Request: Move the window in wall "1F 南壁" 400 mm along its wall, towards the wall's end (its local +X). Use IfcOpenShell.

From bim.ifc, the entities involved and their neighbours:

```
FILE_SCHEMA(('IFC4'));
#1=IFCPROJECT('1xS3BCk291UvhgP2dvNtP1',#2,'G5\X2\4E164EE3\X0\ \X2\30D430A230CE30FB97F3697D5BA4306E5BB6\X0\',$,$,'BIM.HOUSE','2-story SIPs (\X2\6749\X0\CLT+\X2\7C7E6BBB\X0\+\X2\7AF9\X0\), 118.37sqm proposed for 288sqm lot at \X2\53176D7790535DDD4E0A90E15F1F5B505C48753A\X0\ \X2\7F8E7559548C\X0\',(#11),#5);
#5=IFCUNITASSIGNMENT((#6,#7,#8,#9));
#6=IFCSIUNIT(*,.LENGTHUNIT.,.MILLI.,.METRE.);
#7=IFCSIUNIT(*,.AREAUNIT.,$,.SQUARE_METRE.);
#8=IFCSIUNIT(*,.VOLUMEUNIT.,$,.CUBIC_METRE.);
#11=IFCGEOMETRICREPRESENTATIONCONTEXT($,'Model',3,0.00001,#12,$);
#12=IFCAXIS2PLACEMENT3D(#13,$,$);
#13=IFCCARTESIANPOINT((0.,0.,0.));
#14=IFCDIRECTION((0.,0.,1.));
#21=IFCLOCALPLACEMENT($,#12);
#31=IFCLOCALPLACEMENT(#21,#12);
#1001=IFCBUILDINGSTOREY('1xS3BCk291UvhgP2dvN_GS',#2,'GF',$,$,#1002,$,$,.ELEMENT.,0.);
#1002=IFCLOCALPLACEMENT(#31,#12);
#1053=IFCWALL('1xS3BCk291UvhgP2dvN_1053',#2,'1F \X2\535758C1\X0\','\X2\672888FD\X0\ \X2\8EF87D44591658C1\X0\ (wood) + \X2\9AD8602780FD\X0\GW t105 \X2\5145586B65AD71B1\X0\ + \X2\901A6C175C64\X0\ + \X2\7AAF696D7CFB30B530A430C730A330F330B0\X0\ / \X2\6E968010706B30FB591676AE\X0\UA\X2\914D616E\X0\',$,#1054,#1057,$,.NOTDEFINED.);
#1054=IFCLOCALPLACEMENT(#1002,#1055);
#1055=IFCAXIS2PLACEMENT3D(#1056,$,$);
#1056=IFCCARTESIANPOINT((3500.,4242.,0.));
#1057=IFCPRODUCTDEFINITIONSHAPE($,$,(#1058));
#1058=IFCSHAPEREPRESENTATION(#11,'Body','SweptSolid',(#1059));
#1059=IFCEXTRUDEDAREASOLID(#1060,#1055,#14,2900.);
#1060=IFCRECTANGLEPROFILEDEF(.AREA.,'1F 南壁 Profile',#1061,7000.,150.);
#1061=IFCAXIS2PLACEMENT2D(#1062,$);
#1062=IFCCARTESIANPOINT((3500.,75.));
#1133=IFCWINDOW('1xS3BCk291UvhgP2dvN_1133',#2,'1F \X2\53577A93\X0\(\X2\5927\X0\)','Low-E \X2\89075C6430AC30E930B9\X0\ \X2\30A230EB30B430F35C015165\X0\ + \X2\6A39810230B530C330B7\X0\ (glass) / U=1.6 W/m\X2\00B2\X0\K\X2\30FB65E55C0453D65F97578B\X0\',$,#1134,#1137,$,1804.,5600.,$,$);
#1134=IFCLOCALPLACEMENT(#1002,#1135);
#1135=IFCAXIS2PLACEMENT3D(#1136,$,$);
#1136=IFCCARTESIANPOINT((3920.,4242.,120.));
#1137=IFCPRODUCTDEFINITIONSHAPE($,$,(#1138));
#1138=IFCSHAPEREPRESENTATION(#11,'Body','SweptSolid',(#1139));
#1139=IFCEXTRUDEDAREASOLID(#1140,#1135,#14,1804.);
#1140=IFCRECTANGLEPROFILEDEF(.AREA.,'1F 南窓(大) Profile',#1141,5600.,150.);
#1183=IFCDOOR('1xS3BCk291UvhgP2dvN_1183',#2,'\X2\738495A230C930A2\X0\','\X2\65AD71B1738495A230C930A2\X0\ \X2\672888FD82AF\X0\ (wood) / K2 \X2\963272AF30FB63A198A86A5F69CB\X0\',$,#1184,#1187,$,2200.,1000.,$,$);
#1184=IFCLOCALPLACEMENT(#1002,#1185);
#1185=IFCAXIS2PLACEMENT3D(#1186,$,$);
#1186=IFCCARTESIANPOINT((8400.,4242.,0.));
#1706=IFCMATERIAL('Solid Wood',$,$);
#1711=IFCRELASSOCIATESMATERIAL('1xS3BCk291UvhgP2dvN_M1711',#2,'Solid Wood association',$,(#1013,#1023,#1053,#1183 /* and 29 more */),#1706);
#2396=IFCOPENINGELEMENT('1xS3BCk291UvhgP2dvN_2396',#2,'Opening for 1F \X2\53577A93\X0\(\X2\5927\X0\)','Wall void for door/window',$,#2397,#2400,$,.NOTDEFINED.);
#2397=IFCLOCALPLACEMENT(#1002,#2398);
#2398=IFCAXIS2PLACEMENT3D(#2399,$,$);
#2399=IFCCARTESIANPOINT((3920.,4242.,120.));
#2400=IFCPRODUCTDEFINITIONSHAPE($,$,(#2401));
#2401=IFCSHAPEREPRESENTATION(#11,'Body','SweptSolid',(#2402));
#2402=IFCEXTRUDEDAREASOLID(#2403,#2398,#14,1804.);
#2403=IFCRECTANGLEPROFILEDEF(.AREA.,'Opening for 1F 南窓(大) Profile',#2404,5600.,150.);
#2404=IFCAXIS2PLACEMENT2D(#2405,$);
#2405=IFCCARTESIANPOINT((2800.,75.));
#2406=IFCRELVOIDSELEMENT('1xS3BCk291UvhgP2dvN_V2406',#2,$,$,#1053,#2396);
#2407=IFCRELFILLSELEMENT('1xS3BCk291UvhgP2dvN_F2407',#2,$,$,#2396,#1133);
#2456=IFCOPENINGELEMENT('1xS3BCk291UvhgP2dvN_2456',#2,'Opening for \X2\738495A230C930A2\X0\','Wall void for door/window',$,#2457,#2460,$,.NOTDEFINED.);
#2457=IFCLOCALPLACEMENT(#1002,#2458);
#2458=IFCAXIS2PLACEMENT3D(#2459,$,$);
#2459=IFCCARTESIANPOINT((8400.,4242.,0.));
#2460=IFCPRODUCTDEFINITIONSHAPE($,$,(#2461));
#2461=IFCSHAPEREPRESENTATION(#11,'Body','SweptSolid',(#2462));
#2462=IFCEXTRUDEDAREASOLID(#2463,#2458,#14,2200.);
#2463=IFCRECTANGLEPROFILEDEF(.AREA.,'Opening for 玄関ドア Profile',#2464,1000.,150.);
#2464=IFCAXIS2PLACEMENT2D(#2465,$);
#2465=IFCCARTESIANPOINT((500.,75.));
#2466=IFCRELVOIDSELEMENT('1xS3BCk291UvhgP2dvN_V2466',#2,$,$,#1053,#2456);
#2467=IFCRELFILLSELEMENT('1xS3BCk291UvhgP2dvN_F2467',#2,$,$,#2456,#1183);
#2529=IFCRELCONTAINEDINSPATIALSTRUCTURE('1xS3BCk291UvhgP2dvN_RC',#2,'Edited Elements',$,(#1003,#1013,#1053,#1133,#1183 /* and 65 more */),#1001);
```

```python
import ifcopenshell
import ifcopenshell.api.geometry
import ifcopenshell.util.placement

model = ifcopenshell.open("bim.ifc")

window = model.by_guid("1xS3BCk291UvhgP2dvN_1133")
opening = window.FillsVoids[0].RelatingOpeningElement
wall = opening.VoidsElements[0].RelatingBuildingElement

wall_matrix = ifcopenshell.util.placement.get_local_placement(wall.ObjectPlacement)
shift = wall_matrix[:3, 0] * 400.0
before = ifcopenshell.util.placement.get_local_placement(window.ObjectPlacement)[:3, 3].copy()

# The window is not placed relative to its opening, so move both.
for product in (opening, window):
    matrix = ifcopenshell.util.placement.get_local_placement(product.ObjectPlacement)
    matrix[:3, 3] += shift
    ifcopenshell.api.geometry.edit_object_placement(model, product=product, matrix=matrix, is_si=False)

after = ifcopenshell.util.placement.get_local_placement(window.ObjectPlacement)[:3, 3]
print("window moved by", (after - before).round(3) + 0.0)

model.write("bim_v2.ifc")
```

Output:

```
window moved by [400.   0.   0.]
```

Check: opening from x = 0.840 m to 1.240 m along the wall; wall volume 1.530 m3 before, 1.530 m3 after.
